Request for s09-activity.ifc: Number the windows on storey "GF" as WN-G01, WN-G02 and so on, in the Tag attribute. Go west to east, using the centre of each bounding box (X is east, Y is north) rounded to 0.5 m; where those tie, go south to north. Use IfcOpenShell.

First a look at what the model holds.

```python
import ifcopenshell
import ifcopenshell.util.element
import ifcopenshell.util.placement

model = ifcopenshell.open("s09-activity.ifc")
print(model.schema)
storey = next(s for s in model.by_type("IfcBuildingStorey") if s.Name == "GF")
windows = [e for e in ifcopenshell.util.element.get_decomposition(storey) if e.is_a("IfcWindow")]
for e in sorted(windows, key=lambda e: e.id()):
    origin = ifcopenshell.util.placement.get_local_placement(e.ObjectPlacement)[:3, 3]
    print(e.id(), e.Tag, e.Name, origin.round(2) + 0.0, sep=" | ")
```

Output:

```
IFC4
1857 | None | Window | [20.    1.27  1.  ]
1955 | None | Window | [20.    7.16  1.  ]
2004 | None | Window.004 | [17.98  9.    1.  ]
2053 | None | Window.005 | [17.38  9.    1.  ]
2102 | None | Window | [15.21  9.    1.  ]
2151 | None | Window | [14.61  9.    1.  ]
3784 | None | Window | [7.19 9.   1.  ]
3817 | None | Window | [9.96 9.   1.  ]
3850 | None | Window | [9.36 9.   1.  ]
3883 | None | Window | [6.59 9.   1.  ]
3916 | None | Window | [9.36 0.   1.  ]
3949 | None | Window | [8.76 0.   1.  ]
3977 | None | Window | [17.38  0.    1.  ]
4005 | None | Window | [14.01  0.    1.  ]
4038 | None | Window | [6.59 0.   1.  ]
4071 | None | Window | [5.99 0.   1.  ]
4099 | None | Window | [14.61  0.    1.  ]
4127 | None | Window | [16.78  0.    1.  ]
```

```python
import ifcopenshell
import ifcopenshell.geom
import ifcopenshell.util.element
import ifcopenshell.util.shape

model = ifcopenshell.open("s09-activity.ifc")
settings = ifcopenshell.geom.settings()
settings.set("use-world-coords", True)


def centre(element):
    shape = ifcopenshell.geom.create_shape(settings, element)
    return ifcopenshell.util.shape.get_bbox_centroid(shape.geometry)


storey = next(s for s in model.by_type("IfcBuildingStorey") if s.Name == "GF")
windows = [e for e in ifcopenshell.util.element.get_decomposition(storey) if e.is_a("IfcWindow")]

# Insertion points can sit at a corner or the storey origin, so sort by the geometry (in metres).
centres = {e: centre(e) for e in windows}
windows.sort(key=lambda e: (round(centres[e][0] / 0.5), centres[e][1]))

for i, e in enumerate(windows, start=1):
    number = f"WN-G{i:02d}"
    e.Tag = number
    print(e.id(), number)

model.write("s09-activity_v2.ifc")
```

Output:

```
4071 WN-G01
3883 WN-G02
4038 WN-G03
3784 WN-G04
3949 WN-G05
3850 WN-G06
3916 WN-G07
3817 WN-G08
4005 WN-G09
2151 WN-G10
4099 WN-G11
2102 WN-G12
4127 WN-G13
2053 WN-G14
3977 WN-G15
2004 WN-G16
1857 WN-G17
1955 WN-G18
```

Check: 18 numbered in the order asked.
